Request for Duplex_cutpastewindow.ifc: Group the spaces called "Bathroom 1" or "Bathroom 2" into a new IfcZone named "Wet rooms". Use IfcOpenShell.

First a look at what the model holds.

```python
import ifcopenshell

model = ifcopenshell.open("Duplex_cutpastewindow.ifc")
print(model.schema)
seen = {}
for space in model.by_type("IfcSpace"):
    seen[space.LongName] = seen.get(space.LongName, 0) + 1
for name, count in sorted(seen.items(), key=str):
    print(count, "x", name)
print("zones:", [z.Name for z in model.by_type("IfcZone")][:20])
```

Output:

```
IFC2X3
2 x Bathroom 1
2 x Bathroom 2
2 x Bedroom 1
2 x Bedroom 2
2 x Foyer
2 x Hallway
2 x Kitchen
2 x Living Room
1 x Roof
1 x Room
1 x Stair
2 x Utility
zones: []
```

```python
import ifcopenshell
import ifcopenshell.api.group
import ifcopenshell.api.root

model = ifcopenshell.open("Duplex_cutpastewindow.ifc")

names = {"Bathroom 1", "Bathroom 2"}
spaces = [s for s in model.by_type("IfcSpace") if s.LongName in names]

zone = ifcopenshell.api.root.create_entity(model, ifc_class="IfcZone", name="Wet rooms")
ifcopenshell.api.group.assign_group(model, products=spaces, group=zone)
print(len(spaces), "spaces in", zone.Name)

model.write("Duplex_cutpastewindow_rev.ifc")
```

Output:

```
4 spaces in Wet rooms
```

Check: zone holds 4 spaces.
